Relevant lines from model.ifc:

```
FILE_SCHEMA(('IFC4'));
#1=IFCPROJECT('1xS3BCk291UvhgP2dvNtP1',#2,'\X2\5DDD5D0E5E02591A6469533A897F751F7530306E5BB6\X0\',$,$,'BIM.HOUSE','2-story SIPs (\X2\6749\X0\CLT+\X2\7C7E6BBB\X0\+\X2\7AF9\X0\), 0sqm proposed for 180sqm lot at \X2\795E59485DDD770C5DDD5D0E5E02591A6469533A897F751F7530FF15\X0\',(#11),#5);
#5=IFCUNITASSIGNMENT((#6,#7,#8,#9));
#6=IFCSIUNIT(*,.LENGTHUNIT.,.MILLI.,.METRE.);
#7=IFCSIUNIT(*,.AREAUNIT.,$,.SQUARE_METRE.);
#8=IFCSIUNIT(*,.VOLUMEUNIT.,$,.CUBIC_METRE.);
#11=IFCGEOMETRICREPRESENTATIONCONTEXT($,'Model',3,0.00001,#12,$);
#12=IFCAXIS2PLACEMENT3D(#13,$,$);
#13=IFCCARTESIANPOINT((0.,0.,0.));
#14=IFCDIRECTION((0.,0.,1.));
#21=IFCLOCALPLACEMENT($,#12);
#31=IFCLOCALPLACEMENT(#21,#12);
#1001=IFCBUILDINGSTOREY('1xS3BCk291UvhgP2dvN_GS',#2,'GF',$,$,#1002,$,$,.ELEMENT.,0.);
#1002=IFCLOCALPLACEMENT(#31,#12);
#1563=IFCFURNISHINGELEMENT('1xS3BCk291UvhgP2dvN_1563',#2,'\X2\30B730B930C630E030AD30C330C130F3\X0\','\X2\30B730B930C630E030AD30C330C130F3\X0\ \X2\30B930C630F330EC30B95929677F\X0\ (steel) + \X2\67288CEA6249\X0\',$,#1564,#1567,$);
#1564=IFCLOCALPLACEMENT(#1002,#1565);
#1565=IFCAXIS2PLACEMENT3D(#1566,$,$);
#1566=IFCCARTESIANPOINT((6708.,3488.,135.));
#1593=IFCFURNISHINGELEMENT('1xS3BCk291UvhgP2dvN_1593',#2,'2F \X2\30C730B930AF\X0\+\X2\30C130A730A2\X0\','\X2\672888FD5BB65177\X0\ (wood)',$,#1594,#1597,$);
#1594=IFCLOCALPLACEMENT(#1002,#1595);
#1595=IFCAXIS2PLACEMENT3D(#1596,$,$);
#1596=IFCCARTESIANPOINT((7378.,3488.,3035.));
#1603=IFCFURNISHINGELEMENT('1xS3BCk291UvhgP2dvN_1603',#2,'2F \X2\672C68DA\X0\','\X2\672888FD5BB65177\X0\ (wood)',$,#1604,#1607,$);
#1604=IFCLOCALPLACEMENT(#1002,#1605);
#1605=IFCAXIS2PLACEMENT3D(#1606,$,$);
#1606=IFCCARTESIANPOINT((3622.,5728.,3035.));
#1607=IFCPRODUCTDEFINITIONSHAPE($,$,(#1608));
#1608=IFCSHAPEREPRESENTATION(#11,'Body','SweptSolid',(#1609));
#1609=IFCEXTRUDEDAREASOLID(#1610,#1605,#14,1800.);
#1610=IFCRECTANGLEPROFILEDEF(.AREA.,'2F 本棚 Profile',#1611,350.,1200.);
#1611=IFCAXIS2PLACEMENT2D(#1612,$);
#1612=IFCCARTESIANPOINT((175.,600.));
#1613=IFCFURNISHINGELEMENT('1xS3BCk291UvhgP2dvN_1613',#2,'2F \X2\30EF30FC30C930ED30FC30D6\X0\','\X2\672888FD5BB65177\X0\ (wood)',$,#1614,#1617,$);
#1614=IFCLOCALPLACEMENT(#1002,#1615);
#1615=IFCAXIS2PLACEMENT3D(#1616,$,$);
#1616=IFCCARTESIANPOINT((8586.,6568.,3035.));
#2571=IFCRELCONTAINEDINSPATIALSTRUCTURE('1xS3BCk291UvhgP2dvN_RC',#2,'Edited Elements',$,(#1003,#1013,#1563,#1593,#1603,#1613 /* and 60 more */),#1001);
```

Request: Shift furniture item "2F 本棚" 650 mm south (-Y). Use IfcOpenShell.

```python
import ifcopenshell
import ifcopenshell.api.geometry
import ifcopenshell.util.placement
import ifcopenshell.util.unit

model = ifcopenshell.open("model.ifc")
unit_scale = ifcopenshell.util.unit.calculate_unit_scale(model)

item = model.by_guid("1xS3BCk291UvhgP2dvN_1603")
matrix = ifcopenshell.util.placement.get_local_placement(item.ObjectPlacement)
matrix[1, 3] -= 0.65 / unit_scale
ifcopenshell.api.geometry.edit_object_placement(model, product=item, matrix=matrix, is_si=False)

print(ifcopenshell.util.placement.get_local_placement(item.ObjectPlacement).round(3) + 0.0)

model.write("model_updated.ifc")
```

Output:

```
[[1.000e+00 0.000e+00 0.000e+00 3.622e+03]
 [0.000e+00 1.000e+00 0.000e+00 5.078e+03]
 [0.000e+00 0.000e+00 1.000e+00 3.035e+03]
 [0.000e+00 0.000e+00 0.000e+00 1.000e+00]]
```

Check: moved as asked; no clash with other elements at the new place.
